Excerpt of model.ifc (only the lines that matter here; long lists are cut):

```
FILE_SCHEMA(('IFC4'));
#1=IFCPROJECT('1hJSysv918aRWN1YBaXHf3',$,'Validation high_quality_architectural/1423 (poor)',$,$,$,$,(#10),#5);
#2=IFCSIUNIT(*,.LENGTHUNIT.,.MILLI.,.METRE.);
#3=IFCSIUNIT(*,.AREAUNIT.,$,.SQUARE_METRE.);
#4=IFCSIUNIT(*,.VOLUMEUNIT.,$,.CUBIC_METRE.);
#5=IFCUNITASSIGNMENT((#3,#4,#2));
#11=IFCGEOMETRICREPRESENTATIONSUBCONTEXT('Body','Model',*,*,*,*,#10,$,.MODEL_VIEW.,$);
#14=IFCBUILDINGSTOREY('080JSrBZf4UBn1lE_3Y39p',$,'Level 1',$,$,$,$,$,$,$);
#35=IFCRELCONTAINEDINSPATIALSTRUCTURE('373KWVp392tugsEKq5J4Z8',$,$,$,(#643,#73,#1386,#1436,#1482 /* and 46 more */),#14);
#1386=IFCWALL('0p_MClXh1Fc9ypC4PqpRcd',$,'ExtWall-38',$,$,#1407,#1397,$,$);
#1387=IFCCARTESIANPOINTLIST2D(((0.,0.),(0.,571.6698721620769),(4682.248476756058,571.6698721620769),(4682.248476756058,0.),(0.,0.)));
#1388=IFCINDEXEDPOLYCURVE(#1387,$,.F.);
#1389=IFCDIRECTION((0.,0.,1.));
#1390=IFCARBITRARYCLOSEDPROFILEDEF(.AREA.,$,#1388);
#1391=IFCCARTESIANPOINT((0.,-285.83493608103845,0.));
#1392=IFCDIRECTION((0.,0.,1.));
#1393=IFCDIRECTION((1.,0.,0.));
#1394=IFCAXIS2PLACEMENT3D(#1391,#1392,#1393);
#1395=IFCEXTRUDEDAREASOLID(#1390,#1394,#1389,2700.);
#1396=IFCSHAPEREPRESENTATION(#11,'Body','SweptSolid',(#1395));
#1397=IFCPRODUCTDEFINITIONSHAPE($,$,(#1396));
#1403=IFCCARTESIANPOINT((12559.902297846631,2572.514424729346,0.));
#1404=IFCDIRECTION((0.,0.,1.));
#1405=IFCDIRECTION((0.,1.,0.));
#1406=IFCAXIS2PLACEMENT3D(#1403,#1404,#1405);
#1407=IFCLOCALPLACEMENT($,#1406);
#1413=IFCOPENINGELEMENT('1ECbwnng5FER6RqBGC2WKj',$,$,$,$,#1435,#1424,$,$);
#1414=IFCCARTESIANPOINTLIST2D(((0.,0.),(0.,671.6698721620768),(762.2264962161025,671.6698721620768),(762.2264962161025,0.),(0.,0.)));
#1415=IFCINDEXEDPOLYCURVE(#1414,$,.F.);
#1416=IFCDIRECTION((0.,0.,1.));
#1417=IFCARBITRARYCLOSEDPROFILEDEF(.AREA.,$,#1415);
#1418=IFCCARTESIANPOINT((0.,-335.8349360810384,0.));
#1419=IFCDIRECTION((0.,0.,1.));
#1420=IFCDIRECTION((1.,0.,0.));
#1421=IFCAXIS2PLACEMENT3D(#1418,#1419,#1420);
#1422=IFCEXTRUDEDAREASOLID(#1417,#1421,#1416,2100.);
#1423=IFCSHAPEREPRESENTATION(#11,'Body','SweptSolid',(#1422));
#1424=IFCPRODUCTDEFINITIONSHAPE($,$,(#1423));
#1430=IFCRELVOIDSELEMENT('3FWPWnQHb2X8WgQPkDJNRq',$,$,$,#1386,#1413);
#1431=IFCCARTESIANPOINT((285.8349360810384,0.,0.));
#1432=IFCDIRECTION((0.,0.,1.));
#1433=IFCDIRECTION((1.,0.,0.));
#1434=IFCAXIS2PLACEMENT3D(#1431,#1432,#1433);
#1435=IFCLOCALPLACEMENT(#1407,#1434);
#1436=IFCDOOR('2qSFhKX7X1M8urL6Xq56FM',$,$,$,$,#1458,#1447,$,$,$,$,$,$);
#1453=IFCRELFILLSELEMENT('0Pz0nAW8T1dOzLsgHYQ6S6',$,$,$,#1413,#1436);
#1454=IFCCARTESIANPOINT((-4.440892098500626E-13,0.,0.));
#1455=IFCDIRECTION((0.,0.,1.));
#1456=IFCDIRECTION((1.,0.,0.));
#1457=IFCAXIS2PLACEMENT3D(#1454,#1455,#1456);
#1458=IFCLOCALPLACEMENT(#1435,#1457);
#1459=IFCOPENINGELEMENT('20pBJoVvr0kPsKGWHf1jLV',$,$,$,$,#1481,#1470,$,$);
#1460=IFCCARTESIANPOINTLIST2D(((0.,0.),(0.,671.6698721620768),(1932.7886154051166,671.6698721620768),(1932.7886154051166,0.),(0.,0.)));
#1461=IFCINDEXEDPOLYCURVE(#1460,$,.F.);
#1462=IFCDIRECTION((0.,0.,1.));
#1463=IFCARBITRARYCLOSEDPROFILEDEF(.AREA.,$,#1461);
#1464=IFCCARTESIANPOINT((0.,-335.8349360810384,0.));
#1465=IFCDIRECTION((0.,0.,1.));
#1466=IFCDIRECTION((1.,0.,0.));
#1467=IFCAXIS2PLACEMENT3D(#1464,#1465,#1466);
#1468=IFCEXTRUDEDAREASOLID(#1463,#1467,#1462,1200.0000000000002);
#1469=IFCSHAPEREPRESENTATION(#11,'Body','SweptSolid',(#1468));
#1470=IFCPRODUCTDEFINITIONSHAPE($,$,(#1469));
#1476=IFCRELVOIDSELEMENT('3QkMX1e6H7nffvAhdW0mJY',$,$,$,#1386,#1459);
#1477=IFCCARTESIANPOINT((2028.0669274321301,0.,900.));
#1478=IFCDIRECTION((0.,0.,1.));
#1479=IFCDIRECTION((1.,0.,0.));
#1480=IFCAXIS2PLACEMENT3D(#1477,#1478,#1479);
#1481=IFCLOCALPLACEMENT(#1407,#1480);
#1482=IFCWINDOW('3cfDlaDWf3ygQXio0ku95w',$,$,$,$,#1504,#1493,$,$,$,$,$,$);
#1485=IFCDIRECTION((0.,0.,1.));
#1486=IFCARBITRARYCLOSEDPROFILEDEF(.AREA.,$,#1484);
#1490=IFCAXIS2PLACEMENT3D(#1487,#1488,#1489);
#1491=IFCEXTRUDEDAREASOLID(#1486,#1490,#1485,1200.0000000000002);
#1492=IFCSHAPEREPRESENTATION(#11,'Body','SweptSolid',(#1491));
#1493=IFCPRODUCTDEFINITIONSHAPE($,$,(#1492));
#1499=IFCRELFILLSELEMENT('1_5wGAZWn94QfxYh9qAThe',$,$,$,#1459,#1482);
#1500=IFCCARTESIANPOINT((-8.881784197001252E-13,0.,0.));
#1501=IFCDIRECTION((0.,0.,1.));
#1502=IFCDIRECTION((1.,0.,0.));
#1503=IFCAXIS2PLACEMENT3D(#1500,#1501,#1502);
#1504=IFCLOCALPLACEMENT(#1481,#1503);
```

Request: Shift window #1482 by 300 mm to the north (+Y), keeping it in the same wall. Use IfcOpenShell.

```python
import ifcopenshell
import ifcopenshell.api.geometry
import ifcopenshell.util.placement

model = ifcopenshell.open("model.ifc")

window = model.by_id(1482)
opening = window.FillsVoids[0].RelatingOpeningElement
wall = opening.VoidsElements[0].RelatingBuildingElement

wall_matrix = ifcopenshell.util.placement.get_local_placement(wall.ObjectPlacement)
shift = wall_matrix[:3, 0] * 300.0
before = ifcopenshell.util.placement.get_local_placement(window.ObjectPlacement)[:3, 3].copy()

# The window is placed relative to its opening, so it follows when the opening moves.
matrix = ifcopenshell.util.placement.get_local_placement(opening.ObjectPlacement)
matrix[:3, 3] += shift
ifcopenshell.api.geometry.edit_object_placement(
    model, product=opening, matrix=matrix, is_si=False, should_transform_children=True
)

after = ifcopenshell.util.placement.get_local_placement(window.ObjectPlacement)[:3, 3]
print("window moved by", (after - before).round(3) + 0.0)

model.write("model-out.ifc")
```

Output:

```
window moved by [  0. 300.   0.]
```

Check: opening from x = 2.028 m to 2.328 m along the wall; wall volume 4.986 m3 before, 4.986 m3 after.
